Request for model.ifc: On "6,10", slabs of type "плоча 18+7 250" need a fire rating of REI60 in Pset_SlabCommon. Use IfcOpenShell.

First a look at what the model holds.

```python
import ifcopenshell
import ifcopenshell.util.element

model = ifcopenshell.open("model.ifc")
print(model.schema)
storey = next(s for s in model.by_type("IfcBuildingStorey") if s.Name == "6,10")
slabs = [e for e in ifcopenshell.util.element.get_decomposition(storey) if e.is_a("IfcSlab")]
seen = {}
for e in slabs:
    element_type = ifcopenshell.util.element.get_type(e)
    key = (element_type.Name if element_type != e and element_type else None, ifcopenshell.util.element.get_pset(e, "Pset_SlabCommon", "FireRating"))
    seen[key] = seen.get(key, 0) + 1
for (name, value), count in sorted(seen.items(), key=str):
    print(count, "x", name, "|", value)
```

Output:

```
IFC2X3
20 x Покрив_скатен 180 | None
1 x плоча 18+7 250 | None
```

```python
import ifcopenshell
import ifcopenshell.api.pset
import ifcopenshell.util.element

model = ifcopenshell.open("model.ifc")

storey = next(s for s in model.by_type("IfcBuildingStorey") if s.Name == "6,10")
slabs = [e for e in ifcopenshell.util.element.get_decomposition(storey) if e.is_a("IfcSlab")]

count = 0
for e in slabs:
    element_type = ifcopenshell.util.element.get_type(e)
    if element_type in (None, e) or element_type.Name != "плоча 18+7 250":
        continue
    # add_pset returns the element's existing set when there is one.
    pset = ifcopenshell.api.pset.add_pset(model, product=e, name="Pset_SlabCommon")
    ifcopenshell.api.pset.edit_pset(model, pset=pset, properties={"FireRating": "REI60"})
    count += 1

print(count, "slabs updated")

model.write("model-out.ifc")
```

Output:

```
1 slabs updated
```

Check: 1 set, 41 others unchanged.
